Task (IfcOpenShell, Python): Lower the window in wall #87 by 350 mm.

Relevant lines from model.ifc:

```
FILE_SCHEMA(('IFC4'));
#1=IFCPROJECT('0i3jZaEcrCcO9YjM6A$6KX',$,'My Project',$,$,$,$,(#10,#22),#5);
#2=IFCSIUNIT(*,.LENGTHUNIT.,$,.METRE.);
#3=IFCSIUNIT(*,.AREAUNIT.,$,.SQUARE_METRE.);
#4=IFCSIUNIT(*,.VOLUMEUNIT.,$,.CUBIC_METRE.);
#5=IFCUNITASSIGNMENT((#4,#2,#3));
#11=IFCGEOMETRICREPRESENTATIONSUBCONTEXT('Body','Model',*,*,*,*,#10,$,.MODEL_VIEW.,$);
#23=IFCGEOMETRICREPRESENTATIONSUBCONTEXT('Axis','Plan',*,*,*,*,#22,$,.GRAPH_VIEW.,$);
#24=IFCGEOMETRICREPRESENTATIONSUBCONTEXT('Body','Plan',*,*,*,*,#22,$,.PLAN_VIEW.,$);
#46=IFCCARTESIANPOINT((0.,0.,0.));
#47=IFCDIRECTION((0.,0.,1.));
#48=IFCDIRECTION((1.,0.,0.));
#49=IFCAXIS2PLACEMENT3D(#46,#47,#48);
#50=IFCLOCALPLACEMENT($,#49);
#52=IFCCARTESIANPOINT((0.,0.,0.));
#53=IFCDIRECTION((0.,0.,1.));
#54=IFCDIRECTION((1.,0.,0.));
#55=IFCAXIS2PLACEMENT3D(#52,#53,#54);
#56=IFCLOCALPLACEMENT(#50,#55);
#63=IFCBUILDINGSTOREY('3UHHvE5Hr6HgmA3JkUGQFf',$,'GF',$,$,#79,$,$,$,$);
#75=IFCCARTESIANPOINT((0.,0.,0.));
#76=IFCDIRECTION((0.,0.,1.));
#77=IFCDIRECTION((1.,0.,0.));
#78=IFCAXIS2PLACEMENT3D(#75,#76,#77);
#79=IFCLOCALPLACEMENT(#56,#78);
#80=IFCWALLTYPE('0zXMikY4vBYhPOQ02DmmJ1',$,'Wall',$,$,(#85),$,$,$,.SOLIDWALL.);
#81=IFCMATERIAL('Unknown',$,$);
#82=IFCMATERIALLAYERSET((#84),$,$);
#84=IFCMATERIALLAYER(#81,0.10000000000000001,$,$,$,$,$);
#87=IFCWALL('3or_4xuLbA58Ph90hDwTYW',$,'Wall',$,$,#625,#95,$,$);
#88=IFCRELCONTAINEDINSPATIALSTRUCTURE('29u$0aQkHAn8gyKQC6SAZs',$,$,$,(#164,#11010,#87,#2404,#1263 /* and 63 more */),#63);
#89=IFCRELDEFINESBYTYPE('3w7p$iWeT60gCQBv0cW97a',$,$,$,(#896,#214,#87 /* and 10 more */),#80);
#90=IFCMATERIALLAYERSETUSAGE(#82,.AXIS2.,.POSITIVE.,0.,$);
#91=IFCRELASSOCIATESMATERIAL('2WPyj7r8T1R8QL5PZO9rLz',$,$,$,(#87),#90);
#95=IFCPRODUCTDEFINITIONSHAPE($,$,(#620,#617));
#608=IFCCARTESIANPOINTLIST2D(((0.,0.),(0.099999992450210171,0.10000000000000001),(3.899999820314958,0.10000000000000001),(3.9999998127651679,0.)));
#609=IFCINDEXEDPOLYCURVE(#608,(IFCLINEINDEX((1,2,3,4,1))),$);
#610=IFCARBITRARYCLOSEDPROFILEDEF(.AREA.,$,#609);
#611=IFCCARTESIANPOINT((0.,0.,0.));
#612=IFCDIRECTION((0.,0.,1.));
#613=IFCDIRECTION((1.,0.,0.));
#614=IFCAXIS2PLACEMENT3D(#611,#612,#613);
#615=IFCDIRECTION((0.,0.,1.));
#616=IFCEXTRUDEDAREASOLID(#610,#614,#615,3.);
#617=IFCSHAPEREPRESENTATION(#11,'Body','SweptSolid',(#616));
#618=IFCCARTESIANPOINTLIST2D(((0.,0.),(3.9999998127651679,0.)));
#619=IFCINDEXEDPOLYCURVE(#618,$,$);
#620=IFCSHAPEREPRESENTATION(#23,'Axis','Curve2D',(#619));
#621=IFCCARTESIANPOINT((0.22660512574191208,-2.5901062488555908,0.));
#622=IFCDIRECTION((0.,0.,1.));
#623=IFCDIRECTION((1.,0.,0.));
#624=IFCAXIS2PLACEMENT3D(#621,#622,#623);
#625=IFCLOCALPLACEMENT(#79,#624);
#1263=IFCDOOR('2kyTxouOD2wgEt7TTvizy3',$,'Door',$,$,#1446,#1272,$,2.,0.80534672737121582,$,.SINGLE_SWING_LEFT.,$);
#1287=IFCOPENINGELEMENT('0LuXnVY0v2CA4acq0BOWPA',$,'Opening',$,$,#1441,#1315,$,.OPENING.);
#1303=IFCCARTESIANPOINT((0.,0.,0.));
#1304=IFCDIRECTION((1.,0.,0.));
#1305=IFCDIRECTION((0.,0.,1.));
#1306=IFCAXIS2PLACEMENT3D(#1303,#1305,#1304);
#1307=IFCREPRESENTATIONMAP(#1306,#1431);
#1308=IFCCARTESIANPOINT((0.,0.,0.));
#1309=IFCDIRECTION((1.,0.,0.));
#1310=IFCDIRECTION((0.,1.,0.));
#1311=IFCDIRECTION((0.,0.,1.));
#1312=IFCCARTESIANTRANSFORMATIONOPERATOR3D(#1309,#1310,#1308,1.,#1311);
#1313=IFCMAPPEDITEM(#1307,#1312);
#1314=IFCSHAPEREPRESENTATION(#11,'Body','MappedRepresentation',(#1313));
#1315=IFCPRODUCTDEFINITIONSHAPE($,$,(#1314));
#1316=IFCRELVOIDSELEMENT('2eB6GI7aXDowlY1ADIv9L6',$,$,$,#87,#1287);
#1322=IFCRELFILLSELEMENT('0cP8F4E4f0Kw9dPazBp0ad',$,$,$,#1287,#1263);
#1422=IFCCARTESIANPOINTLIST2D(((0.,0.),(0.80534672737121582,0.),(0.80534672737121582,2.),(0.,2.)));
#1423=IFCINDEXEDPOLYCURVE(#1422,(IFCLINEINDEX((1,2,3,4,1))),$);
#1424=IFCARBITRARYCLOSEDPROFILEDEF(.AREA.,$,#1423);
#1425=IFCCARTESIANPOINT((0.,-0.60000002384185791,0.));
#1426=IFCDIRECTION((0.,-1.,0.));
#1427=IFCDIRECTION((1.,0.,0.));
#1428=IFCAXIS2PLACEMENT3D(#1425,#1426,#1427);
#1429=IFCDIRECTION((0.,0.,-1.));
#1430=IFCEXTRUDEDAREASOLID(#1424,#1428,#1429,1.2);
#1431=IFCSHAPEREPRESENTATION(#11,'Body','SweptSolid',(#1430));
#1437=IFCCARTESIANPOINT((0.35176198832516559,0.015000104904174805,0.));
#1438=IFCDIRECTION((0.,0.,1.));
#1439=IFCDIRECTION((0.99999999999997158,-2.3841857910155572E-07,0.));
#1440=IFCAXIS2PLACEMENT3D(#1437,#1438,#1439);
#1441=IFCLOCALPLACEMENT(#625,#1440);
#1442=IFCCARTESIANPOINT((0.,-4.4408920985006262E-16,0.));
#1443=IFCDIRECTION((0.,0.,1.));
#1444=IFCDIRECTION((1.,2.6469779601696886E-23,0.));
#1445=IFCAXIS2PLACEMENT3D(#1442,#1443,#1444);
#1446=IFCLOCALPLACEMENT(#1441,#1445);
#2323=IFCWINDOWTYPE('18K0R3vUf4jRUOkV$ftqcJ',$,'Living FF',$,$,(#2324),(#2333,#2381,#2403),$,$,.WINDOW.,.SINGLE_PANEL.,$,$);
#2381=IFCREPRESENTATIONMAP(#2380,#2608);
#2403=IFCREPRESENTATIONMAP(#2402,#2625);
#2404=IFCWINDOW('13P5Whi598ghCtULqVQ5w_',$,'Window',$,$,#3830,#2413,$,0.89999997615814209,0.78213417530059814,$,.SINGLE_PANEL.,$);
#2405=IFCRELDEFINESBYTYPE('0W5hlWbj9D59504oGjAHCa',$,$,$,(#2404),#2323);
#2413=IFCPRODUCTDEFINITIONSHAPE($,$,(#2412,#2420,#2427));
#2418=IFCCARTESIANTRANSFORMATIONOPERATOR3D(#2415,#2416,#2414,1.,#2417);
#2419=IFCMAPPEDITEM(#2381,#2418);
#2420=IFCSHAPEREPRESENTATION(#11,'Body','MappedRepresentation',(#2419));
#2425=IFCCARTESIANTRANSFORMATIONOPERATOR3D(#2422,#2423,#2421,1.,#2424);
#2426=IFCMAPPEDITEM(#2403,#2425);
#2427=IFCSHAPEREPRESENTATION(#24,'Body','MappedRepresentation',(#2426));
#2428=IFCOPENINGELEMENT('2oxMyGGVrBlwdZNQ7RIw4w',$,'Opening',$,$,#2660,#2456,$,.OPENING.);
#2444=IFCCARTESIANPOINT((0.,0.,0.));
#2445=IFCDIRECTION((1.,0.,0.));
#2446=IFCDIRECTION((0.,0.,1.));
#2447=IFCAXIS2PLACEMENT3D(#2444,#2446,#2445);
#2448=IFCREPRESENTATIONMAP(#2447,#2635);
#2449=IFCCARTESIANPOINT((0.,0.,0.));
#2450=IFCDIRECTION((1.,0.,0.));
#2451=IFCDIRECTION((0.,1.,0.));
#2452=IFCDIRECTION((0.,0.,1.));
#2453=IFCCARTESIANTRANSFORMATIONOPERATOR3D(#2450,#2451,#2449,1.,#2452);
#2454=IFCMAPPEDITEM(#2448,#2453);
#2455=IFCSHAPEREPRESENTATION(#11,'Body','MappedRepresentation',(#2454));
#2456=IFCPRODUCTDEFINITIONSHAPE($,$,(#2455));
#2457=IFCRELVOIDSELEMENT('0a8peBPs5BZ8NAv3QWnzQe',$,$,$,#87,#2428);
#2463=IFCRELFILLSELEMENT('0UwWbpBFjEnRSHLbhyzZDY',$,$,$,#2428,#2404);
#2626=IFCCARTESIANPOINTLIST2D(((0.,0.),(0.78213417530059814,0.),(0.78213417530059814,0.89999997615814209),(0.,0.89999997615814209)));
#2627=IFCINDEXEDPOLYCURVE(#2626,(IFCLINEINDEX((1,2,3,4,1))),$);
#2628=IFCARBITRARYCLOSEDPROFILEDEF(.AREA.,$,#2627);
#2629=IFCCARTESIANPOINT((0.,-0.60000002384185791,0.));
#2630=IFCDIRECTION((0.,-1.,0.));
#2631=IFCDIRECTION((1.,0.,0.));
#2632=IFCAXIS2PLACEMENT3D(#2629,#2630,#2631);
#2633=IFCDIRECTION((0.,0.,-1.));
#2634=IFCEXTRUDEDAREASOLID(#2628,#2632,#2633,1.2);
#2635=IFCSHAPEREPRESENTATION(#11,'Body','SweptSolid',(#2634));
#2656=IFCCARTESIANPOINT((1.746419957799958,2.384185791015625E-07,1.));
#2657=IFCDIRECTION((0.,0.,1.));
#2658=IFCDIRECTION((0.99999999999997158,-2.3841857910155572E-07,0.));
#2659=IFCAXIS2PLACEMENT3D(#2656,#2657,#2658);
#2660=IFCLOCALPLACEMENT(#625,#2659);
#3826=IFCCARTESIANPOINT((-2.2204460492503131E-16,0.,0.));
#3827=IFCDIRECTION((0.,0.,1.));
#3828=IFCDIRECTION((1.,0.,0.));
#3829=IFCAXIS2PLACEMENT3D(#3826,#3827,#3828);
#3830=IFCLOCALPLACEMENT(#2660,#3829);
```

```python
import numpy as np
import ifcopenshell
import ifcopenshell.api.geometry
import ifcopenshell.util.placement
import ifcopenshell.util.unit

model = ifcopenshell.open("model.ifc")
unit_scale = ifcopenshell.util.unit.calculate_unit_scale(model)

window = model.by_id(2404)
opening = window.FillsVoids[0].RelatingOpeningElement
dz = -0.35 / unit_scale

shift = np.array([0.0, 0.0, dz])
# The window is placed relative to its opening, so it follows when the opening moves.
matrix = ifcopenshell.util.placement.get_local_placement(opening.ObjectPlacement)
matrix[:3, 3] += shift
ifcopenshell.api.geometry.edit_object_placement(
    model, product=opening, matrix=matrix, is_si=False, should_transform_children=True
)

print(f"moved by {dz * unit_scale:+.3f} m")

model.write("model_v2.ifc")
```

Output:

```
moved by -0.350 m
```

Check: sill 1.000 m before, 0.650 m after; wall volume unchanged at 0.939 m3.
